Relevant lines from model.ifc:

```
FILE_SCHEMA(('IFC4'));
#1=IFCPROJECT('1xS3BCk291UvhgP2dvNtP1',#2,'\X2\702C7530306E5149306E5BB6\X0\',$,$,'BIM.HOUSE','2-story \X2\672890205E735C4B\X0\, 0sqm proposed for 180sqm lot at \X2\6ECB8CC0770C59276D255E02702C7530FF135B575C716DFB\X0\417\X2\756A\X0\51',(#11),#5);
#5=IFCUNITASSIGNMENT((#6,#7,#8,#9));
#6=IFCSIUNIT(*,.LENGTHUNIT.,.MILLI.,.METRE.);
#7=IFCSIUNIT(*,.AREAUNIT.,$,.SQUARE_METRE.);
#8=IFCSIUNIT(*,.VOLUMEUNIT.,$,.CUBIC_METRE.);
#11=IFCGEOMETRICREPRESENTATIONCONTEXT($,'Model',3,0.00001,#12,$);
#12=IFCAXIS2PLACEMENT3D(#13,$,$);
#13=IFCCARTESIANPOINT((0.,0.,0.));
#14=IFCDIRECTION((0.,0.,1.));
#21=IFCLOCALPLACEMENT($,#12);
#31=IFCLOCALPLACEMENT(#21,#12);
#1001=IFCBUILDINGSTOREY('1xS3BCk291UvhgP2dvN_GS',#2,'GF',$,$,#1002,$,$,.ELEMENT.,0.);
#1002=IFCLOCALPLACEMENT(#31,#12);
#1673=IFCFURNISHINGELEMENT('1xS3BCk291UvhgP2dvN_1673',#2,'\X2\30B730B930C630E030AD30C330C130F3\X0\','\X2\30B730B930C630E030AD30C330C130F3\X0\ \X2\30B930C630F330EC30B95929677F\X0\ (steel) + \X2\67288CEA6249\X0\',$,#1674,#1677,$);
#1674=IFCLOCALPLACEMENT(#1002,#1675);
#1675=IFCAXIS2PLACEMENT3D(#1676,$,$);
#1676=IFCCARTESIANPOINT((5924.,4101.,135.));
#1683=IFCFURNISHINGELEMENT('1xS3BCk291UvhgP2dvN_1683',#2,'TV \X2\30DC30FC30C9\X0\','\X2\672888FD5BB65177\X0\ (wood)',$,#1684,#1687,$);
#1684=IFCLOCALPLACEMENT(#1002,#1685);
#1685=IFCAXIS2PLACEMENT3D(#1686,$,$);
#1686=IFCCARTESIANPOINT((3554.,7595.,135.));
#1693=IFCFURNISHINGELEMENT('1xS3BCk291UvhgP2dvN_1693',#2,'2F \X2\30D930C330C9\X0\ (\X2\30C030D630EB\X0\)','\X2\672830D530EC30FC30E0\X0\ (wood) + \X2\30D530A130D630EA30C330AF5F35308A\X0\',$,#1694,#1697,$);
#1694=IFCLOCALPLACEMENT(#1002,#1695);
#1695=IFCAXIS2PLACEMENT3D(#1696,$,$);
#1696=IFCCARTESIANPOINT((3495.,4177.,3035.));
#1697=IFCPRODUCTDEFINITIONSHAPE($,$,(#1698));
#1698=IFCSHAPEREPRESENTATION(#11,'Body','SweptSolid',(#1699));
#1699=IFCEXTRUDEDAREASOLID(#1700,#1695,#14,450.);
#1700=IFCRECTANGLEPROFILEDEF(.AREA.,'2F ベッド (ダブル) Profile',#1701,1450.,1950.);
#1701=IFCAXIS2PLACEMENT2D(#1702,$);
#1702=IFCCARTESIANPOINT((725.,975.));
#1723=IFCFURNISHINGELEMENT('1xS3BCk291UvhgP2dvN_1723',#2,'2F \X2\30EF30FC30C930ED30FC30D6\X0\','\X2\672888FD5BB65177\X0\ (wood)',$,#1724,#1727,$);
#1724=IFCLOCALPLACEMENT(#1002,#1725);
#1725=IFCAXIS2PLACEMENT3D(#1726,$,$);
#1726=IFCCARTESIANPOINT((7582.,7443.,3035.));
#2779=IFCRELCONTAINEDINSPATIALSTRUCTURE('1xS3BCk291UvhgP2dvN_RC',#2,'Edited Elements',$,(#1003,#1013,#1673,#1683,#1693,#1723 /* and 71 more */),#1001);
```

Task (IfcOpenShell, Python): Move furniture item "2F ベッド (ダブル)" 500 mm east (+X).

```python
import ifcopenshell
import ifcopenshell.api.geometry
import ifcopenshell.util.placement
import ifcopenshell.util.unit

model = ifcopenshell.open("model.ifc")
unit_scale = ifcopenshell.util.unit.calculate_unit_scale(model)

item = model.by_guid("1xS3BCk291UvhgP2dvN_1693")
matrix = ifcopenshell.util.placement.get_local_placement(item.ObjectPlacement)
matrix[0, 3] += 0.5 / unit_scale
ifcopenshell.api.geometry.edit_object_placement(model, product=item, matrix=matrix, is_si=False)

print(ifcopenshell.util.placement.get_local_placement(item.ObjectPlacement).round(3) + 0.0)

model.write("model-out.ifc")
```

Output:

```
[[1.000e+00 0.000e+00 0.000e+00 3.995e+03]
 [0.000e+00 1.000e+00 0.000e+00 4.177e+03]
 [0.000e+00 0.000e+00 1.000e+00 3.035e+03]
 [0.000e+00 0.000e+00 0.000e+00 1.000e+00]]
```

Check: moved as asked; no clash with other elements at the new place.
